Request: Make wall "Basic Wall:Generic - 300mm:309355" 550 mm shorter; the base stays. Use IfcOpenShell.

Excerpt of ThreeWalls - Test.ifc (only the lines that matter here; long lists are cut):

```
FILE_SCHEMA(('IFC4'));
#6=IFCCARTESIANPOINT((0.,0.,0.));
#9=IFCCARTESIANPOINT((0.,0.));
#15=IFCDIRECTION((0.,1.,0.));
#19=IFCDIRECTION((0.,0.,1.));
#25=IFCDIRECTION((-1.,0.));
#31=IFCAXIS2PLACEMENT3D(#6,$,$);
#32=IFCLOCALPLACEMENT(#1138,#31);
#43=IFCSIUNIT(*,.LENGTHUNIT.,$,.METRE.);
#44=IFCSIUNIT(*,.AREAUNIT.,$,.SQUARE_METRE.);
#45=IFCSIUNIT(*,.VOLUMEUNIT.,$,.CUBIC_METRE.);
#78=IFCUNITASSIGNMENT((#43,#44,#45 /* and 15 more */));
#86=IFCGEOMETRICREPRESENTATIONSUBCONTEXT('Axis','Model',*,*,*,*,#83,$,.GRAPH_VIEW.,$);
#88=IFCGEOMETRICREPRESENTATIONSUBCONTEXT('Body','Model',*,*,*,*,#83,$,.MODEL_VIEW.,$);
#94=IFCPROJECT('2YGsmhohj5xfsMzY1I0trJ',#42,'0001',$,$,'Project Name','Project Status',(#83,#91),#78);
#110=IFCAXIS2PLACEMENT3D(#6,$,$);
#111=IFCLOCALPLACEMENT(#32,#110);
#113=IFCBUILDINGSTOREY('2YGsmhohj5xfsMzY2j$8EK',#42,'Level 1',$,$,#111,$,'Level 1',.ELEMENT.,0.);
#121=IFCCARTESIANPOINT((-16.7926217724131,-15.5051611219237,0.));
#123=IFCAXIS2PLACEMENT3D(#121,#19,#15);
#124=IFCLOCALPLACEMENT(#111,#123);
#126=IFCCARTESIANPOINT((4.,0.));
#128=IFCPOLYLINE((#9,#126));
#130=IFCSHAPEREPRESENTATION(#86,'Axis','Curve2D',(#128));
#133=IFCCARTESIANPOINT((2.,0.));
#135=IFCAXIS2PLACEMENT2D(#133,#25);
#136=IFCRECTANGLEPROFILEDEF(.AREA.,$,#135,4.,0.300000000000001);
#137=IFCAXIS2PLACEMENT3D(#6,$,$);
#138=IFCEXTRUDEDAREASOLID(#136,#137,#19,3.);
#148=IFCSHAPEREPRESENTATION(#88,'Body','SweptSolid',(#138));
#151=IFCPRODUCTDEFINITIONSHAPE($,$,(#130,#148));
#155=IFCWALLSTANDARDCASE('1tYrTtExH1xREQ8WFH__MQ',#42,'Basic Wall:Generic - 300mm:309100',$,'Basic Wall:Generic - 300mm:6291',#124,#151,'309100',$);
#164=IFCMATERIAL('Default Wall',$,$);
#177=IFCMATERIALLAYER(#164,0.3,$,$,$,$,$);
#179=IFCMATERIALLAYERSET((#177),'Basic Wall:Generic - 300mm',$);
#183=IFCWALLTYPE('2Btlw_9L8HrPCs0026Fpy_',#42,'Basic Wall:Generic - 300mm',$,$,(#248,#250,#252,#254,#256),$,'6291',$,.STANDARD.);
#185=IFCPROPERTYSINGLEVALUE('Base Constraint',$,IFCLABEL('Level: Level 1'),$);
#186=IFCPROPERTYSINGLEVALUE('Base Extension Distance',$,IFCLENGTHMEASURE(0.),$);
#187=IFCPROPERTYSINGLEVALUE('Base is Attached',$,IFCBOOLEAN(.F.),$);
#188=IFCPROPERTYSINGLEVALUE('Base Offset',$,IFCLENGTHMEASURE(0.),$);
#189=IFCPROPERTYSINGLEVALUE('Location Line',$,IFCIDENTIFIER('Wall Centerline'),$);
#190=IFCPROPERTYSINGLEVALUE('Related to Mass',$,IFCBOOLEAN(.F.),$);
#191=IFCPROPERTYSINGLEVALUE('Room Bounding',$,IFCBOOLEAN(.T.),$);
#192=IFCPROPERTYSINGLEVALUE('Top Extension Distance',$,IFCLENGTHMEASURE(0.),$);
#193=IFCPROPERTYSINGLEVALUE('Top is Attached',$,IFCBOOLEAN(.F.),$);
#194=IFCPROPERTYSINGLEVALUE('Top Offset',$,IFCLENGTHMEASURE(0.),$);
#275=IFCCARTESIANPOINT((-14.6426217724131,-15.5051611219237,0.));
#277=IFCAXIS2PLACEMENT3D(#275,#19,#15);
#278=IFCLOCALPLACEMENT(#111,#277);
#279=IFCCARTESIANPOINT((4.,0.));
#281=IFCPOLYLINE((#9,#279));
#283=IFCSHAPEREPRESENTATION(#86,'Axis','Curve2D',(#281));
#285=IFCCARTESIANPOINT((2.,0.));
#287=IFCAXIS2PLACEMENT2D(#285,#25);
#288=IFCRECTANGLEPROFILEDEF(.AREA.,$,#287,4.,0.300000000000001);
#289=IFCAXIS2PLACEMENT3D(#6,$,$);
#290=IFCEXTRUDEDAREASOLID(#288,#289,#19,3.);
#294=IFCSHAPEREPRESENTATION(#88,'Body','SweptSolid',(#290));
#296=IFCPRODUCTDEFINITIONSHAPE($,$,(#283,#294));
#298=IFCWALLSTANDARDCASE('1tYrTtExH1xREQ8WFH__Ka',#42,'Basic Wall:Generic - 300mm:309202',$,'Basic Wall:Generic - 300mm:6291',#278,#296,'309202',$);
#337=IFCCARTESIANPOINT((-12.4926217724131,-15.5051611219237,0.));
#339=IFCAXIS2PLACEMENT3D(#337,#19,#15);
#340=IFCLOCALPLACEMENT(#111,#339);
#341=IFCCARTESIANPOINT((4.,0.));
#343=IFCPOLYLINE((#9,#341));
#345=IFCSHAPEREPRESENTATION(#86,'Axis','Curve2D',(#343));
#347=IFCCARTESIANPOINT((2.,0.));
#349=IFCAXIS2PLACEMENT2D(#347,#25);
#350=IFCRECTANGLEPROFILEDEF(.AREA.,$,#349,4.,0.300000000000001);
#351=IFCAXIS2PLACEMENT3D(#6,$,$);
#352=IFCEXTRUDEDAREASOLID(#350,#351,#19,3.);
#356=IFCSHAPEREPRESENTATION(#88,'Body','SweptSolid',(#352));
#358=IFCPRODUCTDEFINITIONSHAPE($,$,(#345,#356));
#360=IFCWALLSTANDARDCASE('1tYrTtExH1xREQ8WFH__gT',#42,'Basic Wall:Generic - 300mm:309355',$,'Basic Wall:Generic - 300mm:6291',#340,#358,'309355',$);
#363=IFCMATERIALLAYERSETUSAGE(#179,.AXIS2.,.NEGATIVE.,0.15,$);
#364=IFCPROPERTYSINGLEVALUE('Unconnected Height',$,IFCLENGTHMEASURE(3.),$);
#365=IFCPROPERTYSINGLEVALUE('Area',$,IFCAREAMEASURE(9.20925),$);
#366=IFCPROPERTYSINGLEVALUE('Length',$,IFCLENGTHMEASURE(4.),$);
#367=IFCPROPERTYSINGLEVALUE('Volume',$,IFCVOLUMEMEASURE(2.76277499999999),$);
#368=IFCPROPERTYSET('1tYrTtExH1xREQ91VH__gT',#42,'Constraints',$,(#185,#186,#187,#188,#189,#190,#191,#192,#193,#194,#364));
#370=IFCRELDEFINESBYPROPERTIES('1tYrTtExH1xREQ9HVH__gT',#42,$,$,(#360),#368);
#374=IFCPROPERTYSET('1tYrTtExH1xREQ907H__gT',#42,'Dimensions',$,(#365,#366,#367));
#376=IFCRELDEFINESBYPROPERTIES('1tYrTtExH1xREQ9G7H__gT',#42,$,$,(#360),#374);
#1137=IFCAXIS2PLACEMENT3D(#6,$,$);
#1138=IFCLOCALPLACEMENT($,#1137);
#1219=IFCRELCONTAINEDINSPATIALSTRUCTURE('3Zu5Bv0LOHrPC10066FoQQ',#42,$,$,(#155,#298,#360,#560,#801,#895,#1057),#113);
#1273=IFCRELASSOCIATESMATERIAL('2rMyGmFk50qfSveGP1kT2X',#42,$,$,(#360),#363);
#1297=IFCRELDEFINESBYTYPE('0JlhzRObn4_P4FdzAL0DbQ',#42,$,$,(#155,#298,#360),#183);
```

```python
import ifcopenshell
import ifcopenshell.api.pset
import ifcopenshell.geom
import ifcopenshell.util.element
import ifcopenshell.util.representation
import ifcopenshell.util.shape
import ifcopenshell.util.unit

model = ifcopenshell.open("ThreeWalls - Test.ifc")
area_scale = ifcopenshell.util.unit.calculate_unit_scale(model, "AREAUNIT")
volume_scale = ifcopenshell.util.unit.calculate_unit_scale(model, "VOLUMEUNIT")
settings = ifcopenshell.geom.settings()


def volume(element):
    """Net volume in cubic metres, openings subtracted."""
    shape = ifcopenshell.geom.create_shape(settings, element)
    return ifcopenshell.util.shape.get_volume(shape.geometry)


wall = model.by_guid("1tYrTtExH1xREQ8WFH__gT")
before = volume(wall)

body = ifcopenshell.util.representation.get_representation(wall, "Model", "Body")
solid = body.Items[0]
old_height = solid.Depth
solid.Depth -= 0.55
after = volume(wall)
thickness = 0.3  # wall thickness in metres

# Update the stored height, areas and volumes.
pset = model.by_id(ifcopenshell.util.element.get_pset(wall, "Constraints", should_inherit=False)["id"])
ifcopenshell.api.pset.edit_pset(model, pset=pset, properties={
    "Unconnected Height": model.create_entity("IfcLengthMeasure", solid.Depth),
})
pset = model.by_id(ifcopenshell.util.element.get_pset(wall, "Dimensions", should_inherit=False)["id"])
ifcopenshell.api.pset.edit_pset(model, pset=pset, properties={
    "Area": model.create_entity("IfcAreaMeasure", after / thickness / area_scale),
    "Volume": model.create_entity("IfcVolumeMeasure", after / volume_scale),
})

print(f"height {old_height:g} -> {solid.Depth:g}, volume {before:.3f} -> {after:.3f} m3")

model.write("ThreeWalls - Test_v2.ifc")
```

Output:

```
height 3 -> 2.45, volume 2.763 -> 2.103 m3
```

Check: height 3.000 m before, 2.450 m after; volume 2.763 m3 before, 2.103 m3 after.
